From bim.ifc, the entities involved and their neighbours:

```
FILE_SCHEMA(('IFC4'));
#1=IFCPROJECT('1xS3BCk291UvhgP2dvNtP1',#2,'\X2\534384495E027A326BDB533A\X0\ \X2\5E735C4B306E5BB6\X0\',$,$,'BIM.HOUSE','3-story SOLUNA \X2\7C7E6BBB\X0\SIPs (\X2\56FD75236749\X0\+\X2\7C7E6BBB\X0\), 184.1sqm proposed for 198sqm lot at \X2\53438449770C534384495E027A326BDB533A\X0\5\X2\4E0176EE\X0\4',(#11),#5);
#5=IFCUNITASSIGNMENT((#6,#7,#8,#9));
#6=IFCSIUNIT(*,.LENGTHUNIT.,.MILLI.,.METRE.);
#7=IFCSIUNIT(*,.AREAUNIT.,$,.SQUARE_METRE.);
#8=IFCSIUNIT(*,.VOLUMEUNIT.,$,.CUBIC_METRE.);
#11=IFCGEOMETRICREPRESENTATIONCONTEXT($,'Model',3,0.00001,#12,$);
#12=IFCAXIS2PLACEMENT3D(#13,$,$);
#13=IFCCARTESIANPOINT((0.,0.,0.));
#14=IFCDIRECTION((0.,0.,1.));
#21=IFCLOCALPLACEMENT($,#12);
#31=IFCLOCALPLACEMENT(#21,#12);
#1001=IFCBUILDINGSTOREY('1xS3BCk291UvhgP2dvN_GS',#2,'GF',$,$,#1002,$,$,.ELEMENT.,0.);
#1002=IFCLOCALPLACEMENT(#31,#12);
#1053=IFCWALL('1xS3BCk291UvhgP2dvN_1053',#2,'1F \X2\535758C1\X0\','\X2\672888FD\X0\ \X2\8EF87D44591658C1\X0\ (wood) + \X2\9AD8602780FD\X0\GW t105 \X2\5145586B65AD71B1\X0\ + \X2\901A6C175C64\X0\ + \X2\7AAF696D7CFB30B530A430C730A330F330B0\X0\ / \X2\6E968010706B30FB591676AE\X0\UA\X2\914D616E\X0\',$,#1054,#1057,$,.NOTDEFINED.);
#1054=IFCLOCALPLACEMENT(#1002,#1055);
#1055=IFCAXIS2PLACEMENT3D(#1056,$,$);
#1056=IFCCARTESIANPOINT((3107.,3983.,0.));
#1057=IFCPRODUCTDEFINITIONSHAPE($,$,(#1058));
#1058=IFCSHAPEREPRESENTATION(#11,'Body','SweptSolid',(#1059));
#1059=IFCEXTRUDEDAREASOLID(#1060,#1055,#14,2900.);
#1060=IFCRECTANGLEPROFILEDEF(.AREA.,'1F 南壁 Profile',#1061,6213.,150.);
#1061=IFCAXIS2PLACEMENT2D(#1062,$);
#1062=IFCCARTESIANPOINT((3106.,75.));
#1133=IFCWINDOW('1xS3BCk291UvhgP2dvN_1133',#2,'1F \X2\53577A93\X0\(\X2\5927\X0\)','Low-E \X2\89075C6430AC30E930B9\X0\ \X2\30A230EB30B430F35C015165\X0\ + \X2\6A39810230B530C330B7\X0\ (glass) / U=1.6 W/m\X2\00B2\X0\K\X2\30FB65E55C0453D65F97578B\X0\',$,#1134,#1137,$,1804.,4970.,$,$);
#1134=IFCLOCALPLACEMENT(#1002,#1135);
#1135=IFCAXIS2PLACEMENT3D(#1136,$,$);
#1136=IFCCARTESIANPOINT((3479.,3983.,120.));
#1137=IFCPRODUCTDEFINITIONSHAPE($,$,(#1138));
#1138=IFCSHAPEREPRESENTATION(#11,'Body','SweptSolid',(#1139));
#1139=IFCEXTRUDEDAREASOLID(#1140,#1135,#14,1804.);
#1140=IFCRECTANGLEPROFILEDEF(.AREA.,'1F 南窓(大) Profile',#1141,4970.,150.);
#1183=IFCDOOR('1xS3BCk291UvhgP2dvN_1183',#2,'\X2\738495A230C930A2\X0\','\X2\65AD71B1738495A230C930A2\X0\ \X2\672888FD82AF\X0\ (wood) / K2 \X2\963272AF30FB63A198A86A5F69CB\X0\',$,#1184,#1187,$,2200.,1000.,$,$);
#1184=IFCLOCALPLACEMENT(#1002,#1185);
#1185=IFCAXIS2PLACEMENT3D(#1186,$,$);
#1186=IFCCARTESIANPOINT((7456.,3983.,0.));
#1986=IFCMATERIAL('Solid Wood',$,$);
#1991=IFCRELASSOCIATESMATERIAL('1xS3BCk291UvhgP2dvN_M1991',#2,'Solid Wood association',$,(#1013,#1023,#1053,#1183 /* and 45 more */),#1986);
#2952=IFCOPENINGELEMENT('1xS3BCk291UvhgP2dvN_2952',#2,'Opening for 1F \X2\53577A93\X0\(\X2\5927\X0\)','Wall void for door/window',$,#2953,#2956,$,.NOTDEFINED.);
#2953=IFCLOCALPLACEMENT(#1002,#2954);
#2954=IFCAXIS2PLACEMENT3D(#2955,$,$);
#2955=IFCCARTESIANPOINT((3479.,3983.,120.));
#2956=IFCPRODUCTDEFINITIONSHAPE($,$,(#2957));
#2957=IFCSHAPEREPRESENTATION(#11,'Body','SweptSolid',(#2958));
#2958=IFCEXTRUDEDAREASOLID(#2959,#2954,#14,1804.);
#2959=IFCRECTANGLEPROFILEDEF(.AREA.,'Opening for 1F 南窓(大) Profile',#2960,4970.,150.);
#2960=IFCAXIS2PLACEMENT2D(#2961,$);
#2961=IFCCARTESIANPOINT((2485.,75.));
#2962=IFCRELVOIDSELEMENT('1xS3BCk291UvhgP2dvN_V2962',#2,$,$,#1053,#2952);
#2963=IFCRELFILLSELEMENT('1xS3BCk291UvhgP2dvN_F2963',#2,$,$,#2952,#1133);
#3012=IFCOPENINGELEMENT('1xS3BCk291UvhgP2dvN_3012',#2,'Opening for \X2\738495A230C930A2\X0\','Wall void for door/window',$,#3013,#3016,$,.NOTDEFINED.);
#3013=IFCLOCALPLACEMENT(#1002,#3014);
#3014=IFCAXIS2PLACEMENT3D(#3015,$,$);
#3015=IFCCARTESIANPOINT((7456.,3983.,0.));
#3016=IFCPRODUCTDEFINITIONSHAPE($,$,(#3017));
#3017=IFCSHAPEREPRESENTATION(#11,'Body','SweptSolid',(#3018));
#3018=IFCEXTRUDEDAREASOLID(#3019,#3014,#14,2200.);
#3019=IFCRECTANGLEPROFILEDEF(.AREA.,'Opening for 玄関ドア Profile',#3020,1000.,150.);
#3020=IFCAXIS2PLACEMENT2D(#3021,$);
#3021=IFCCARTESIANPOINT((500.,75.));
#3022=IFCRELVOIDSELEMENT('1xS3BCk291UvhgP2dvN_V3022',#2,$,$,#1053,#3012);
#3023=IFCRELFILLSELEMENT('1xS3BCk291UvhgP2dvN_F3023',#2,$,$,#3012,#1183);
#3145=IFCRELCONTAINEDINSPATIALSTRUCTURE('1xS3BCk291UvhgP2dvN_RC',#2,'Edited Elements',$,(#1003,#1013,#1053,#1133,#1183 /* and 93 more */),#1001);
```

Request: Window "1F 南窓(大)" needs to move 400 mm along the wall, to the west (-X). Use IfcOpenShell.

```python
import ifcopenshell
import ifcopenshell.api.geometry
import ifcopenshell.util.placement
import ifcopenshell.util.unit

model = ifcopenshell.open("bim.ifc")
unit_scale = ifcopenshell.util.unit.calculate_unit_scale(model)

window = model.by_id(1133)
opening = window.FillsVoids[0].RelatingOpeningElement
wall = opening.VoidsElements[0].RelatingBuildingElement

wall_matrix = ifcopenshell.util.placement.get_local_placement(wall.ObjectPlacement)
shift = wall_matrix[:3, 0] * -0.4 / unit_scale
before = ifcopenshell.util.placement.get_local_placement(window.ObjectPlacement)[:3, 3].copy()

# The window is not placed relative to its opening, so move both.
for product in (opening, window):
    matrix = ifcopenshell.util.placement.get_local_placement(product.ObjectPlacement)
    matrix[:3, 3] += shift
    ifcopenshell.api.geometry.edit_object_placement(model, product=product, matrix=matrix, is_si=False)

after = ifcopenshell.util.placement.get_local_placement(window.ObjectPlacement)[:3, 3]
print("window moved by", (after - before).round(3) + 0.0)

model.write("bim_v2.ifc")
```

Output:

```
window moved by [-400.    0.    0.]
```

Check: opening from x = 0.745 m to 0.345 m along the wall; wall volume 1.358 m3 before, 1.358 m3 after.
